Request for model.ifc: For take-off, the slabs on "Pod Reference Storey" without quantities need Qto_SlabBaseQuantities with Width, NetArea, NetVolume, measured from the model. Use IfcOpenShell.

First a look at what the model holds.

```python
import ifcopenshell
import ifcopenshell.util.element
import ifcopenshell.util.unit

model = ifcopenshell.open("model.ifc")
print(model.schema)
for unit_type in ("LENGTHUNIT", "AREAUNIT", "VOLUMEUNIT"):
    print(unit_type, ifcopenshell.util.unit.calculate_unit_scale(model, unit_type))
storey = next(s for s in model.by_type("IfcBuildingStorey") if s.Name == "Pod Reference Storey")
slabs = [e for e in ifcopenshell.util.element.get_decomposition(storey) if e.is_a("IfcSlab")]
for e in sorted(slabs, key=lambda e: e.id()):
    print(e.id(), e.is_a(), e.Name, list(ifcopenshell.util.element.get_psets(e, qtos_only=True)), sep=" | ")
```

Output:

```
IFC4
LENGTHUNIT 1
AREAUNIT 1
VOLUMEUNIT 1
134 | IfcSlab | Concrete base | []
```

```python
import ifcopenshell
import ifcopenshell.api.pset
import ifcopenshell.geom
import ifcopenshell.util.element
import ifcopenshell.util.shape
import ifcopenshell.util.unit

model = ifcopenshell.open("model.ifc")
unit_scale = ifcopenshell.util.unit.calculate_unit_scale(model)
area_scale = ifcopenshell.util.unit.calculate_unit_scale(model, "AREAUNIT")
volume_scale = ifcopenshell.util.unit.calculate_unit_scale(model, "VOLUMEUNIT")
settings = ifcopenshell.geom.settings()

storey = next(s for s in model.by_type("IfcBuildingStorey") if s.Name == "Pod Reference Storey")
slabs = [e for e in ifcopenshell.util.element.get_decomposition(storey) if e.is_a("IfcSlab")]

for e in sorted(slabs, key=lambda e: e.id()):
    if ifcopenshell.util.element.get_psets(e, qtos_only=True, should_inherit=False):
        continue
    # Geometry comes back in metres, in the element's own axes.
    shape = ifcopenshell.geom.create_shape(settings, e)
    values = {
        "Width": ifcopenshell.util.shape.get_z(shape.geometry) / unit_scale,
        "NetArea": ifcopenshell.util.shape.get_footprint_area(shape.geometry) / area_scale,
        "NetVolume": ifcopenshell.util.shape.get_volume(shape.geometry) / volume_scale,
    }
    qto = ifcopenshell.api.pset.add_qto(model, product=e, name="Qto_SlabBaseQuantities")
    ifcopenshell.api.pset.edit_qto(model, qto=qto, properties=values)
    print(e.id(), {k: round(v, 3) for k, v in values.items()})

model.write("model_v2.ifc")
```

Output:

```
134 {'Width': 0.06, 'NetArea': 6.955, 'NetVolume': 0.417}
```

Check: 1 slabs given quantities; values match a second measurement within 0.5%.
